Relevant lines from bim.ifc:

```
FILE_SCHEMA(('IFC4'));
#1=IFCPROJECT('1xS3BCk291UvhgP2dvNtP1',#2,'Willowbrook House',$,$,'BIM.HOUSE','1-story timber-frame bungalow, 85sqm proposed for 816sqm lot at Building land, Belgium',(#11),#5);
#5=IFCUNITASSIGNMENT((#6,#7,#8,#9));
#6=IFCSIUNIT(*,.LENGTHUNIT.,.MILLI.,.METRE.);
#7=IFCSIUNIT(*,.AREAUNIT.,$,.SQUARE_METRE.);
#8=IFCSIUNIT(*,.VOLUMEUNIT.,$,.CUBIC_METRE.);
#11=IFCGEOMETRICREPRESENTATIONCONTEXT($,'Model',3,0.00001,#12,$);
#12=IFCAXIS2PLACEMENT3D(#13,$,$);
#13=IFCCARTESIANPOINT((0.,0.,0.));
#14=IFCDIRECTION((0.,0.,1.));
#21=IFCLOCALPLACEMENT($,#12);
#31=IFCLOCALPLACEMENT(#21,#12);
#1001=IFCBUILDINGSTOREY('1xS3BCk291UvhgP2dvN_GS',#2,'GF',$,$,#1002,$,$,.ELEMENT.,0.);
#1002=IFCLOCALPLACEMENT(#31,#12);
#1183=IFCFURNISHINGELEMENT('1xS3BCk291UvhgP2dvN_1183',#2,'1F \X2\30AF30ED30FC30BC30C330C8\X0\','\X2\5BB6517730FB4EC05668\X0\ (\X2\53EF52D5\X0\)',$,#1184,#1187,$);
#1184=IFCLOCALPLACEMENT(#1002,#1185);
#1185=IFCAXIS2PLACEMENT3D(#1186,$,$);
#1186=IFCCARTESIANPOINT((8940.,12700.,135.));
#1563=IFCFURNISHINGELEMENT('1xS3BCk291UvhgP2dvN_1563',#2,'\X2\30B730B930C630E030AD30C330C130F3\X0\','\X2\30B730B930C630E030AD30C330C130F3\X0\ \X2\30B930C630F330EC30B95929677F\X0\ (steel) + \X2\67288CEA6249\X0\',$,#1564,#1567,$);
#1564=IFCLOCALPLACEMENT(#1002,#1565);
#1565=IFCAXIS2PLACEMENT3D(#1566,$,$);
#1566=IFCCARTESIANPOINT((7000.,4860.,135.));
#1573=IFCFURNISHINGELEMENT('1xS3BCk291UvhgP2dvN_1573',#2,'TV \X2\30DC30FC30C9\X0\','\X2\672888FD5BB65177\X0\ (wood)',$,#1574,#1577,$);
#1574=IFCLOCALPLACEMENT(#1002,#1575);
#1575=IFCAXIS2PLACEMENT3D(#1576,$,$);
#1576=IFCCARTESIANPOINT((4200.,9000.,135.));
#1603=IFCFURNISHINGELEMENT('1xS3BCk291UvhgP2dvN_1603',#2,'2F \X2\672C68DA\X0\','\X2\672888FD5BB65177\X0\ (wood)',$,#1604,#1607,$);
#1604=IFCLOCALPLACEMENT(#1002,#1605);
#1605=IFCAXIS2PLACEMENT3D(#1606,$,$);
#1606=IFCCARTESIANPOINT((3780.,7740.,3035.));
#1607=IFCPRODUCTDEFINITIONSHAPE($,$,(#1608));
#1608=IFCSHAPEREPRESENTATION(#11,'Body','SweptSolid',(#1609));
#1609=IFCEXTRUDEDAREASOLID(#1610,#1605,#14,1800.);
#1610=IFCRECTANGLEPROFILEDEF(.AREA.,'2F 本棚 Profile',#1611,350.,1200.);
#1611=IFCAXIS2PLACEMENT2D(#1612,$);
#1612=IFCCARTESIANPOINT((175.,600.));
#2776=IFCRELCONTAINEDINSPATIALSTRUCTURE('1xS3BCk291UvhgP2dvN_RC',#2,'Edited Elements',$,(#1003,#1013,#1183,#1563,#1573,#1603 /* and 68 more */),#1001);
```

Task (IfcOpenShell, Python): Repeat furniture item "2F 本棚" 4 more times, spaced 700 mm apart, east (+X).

```python
import numpy as np
import ifcopenshell
import ifcopenshell.api.geometry
import ifcopenshell.api.root
import ifcopenshell.util.element
import ifcopenshell.util.placement

model = ifcopenshell.open("bim.ifc")


def reuse_history(source, copy):
    """copy_class also copies each property set's owner history, people and application; keep the originals."""
    for rel in copy.IsDefinedBy:
        if rel.is_a("IfcRelDefinesByProperties") and (history := rel.RelatingPropertyDefinition.OwnerHistory):
            rel.RelatingPropertyDefinition.OwnerHistory = source.OwnerHistory
            ifcopenshell.util.element.remove_deep2(model, history)


source = model.by_id(1603)
base = ifcopenshell.util.placement.get_local_placement(source.ObjectPlacement)
step = np.array([1.0, 0.0, 0.0]) * 700.0

for i in range(1, 5):
    copy = ifcopenshell.api.root.copy_class(model, product=source)
    copy.Representation = ifcopenshell.util.element.copy_deep(
        model, source.Representation, exclude=["IfcGeometricRepresentationContext", "IfcRepresentationMap"]
    )
    reuse_history(source, copy)
    matrix = base.copy()
    matrix[:3, 3] += i * step
    print("added at", matrix[:3, 3].round(3) + 0.0)
    ifcopenshell.api.geometry.edit_object_placement(model, product=copy, matrix=matrix, is_si=False)

model.write("bim_rev.ifc")
```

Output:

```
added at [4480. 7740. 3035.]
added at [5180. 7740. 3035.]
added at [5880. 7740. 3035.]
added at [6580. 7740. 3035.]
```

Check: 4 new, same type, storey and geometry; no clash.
